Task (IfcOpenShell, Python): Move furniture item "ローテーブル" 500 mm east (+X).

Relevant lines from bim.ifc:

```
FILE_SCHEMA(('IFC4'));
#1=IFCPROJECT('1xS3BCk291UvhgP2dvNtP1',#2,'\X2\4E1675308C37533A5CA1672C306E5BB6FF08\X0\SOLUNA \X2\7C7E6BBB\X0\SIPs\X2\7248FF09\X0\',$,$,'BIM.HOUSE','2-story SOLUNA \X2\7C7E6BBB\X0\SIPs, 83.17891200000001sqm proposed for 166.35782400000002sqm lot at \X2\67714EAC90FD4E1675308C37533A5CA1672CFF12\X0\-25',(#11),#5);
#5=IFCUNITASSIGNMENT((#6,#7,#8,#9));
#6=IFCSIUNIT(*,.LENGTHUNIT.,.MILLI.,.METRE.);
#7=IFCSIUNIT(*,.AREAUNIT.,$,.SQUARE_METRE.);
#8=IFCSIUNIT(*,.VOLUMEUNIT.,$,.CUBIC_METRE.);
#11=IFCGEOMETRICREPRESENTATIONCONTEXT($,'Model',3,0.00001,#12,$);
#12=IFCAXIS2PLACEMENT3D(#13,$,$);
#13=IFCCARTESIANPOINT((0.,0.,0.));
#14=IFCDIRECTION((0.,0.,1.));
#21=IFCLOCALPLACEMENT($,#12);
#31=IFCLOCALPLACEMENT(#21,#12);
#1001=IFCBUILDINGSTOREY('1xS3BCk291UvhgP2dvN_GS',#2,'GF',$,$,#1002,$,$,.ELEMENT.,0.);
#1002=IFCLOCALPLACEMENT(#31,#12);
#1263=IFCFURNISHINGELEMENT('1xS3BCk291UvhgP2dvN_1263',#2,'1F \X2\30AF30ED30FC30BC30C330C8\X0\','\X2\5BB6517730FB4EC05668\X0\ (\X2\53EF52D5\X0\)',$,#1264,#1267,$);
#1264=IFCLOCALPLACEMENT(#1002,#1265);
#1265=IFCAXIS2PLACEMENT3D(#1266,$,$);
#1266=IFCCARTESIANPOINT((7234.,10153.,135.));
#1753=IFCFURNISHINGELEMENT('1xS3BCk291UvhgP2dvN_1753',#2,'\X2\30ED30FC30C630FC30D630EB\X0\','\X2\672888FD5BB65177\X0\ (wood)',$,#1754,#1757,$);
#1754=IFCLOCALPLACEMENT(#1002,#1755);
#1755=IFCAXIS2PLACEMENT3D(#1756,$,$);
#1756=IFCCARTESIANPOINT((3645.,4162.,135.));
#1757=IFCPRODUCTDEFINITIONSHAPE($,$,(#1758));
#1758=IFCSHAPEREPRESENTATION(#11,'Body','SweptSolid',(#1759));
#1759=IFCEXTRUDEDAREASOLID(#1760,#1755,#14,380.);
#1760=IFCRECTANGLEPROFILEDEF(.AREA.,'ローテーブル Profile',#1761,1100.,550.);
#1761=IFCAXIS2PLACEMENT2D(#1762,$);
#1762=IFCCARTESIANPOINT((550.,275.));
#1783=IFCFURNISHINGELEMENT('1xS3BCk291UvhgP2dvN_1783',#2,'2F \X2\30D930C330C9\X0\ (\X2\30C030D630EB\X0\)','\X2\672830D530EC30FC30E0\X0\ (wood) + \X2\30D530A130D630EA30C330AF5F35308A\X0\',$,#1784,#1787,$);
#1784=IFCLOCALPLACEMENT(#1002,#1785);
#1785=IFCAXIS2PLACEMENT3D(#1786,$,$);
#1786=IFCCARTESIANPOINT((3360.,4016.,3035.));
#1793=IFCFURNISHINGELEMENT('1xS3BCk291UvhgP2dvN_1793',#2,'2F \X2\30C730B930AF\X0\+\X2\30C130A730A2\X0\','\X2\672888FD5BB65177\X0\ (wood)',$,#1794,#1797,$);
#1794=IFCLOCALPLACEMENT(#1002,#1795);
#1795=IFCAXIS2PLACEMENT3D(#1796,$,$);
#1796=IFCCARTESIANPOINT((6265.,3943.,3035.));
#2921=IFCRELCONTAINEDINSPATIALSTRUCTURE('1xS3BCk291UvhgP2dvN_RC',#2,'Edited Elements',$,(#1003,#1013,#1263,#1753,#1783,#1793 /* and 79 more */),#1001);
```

```python
import ifcopenshell
import ifcopenshell.api.geometry
import ifcopenshell.util.placement
import ifcopenshell.util.unit

model = ifcopenshell.open("bim.ifc")
unit_scale = ifcopenshell.util.unit.calculate_unit_scale(model)

item = model.by_guid("1xS3BCk291UvhgP2dvN_1753")
matrix = ifcopenshell.util.placement.get_local_placement(item.ObjectPlacement)
matrix[0, 3] += 0.5 / unit_scale
ifcopenshell.api.geometry.edit_object_placement(model, product=item, matrix=matrix, is_si=False)

print(ifcopenshell.util.placement.get_local_placement(item.ObjectPlacement).round(3) + 0.0)

model.write("bim_rev.ifc")
```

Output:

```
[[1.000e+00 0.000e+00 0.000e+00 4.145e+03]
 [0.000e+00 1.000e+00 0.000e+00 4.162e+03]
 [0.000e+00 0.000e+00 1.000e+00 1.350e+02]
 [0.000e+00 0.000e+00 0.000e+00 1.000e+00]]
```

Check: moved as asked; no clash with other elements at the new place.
